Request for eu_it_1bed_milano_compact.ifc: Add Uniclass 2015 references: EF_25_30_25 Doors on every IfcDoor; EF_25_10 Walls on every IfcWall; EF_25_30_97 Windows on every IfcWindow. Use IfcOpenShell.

First a look at what the model holds.

```python
import ifcopenshell

model = ifcopenshell.open("eu_it_1bed_milano_compact.ifc")
print(model.schema)
print("classifications:", [c.Name for c in model.by_type("IfcClassification")])
for ifc_class in ("IfcDoor", "IfcRoof", "IfcStair", "IfcWall", "IfcWindow"):
    print(ifc_class, len(model.by_type(ifc_class)))
```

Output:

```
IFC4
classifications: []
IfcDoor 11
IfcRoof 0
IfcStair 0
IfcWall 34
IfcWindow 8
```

```python
import ifcopenshell
import ifcopenshell.api.classification

model = ifcopenshell.open("eu_it_1bed_milano_compact.ifc")

system = ifcopenshell.api.classification.add_classification(model, classification="Uniclass 2015")

codes = {
    "IfcDoor": ("EF_25_30_25", "Doors"),
    "IfcWall": ("EF_25_10", "Walls"),
    "IfcWindow": ("EF_25_30_97", "Windows"),
}
for ifc_class, (code, name) in codes.items():
    products = model.by_type(ifc_class)
    ifcopenshell.api.classification.add_reference(
        model, products=products, classification=system, identification=code, name=name
    )
    print(code, len(products))

model.write("eu_it_1bed_milano_compact_edited.ifc")
```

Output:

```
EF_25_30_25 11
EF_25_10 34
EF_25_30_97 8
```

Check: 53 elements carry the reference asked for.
